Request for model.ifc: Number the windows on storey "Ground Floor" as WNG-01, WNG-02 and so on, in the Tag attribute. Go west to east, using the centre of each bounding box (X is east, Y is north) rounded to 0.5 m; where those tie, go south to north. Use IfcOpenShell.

First a look at what the model holds.

```python
import ifcopenshell
import ifcopenshell.util.element
import ifcopenshell.util.placement

model = ifcopenshell.open("model.ifc")
print(model.schema)
storey = next(s for s in model.by_type("IfcBuildingStorey") if s.Name == "Ground Floor")
windows = [e for e in ifcopenshell.util.element.get_decomposition(storey) if e.is_a("IfcWindow")]
for e in sorted(windows, key=lambda e: e.id()):
    origin = ifcopenshell.util.placement.get_local_placement(e.ObjectPlacement)[:3, 3]
    print(e.id(), e.Tag, e.Name, origin.round(2) + 0.0, sep=" | ")
```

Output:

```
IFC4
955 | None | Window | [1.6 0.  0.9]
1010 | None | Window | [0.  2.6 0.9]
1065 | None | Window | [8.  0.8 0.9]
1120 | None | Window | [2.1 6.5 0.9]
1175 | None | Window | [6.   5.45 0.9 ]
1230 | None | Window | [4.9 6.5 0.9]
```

```python
import ifcopenshell
import ifcopenshell.geom
import ifcopenshell.util.element
import ifcopenshell.util.shape

model = ifcopenshell.open("model.ifc")
settings = ifcopenshell.geom.settings()
settings.set("use-world-coords", True)


def centre(element):
    shape = ifcopenshell.geom.create_shape(settings, element)
    return ifcopenshell.util.shape.get_bbox_centroid(shape.geometry)


storey = next(s for s in model.by_type("IfcBuildingStorey") if s.Name == "Ground Floor")
windows = [e for e in ifcopenshell.util.element.get_decomposition(storey) if e.is_a("IfcWindow")]

# Insertion points can sit at a corner or the storey origin, so sort by the geometry (in metres).
centres = {e: centre(e) for e in windows}
windows.sort(key=lambda e: (round(centres[e][0] / 0.5), centres[e][1]))

for i, e in enumerate(windows, start=1):
    number = f"WNG-{i:02d}"
    e.Tag = number
    print(e.id(), number)

model.write("model_edited.ifc")
```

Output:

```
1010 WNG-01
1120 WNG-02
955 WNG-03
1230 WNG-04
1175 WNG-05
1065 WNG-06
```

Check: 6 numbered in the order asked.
